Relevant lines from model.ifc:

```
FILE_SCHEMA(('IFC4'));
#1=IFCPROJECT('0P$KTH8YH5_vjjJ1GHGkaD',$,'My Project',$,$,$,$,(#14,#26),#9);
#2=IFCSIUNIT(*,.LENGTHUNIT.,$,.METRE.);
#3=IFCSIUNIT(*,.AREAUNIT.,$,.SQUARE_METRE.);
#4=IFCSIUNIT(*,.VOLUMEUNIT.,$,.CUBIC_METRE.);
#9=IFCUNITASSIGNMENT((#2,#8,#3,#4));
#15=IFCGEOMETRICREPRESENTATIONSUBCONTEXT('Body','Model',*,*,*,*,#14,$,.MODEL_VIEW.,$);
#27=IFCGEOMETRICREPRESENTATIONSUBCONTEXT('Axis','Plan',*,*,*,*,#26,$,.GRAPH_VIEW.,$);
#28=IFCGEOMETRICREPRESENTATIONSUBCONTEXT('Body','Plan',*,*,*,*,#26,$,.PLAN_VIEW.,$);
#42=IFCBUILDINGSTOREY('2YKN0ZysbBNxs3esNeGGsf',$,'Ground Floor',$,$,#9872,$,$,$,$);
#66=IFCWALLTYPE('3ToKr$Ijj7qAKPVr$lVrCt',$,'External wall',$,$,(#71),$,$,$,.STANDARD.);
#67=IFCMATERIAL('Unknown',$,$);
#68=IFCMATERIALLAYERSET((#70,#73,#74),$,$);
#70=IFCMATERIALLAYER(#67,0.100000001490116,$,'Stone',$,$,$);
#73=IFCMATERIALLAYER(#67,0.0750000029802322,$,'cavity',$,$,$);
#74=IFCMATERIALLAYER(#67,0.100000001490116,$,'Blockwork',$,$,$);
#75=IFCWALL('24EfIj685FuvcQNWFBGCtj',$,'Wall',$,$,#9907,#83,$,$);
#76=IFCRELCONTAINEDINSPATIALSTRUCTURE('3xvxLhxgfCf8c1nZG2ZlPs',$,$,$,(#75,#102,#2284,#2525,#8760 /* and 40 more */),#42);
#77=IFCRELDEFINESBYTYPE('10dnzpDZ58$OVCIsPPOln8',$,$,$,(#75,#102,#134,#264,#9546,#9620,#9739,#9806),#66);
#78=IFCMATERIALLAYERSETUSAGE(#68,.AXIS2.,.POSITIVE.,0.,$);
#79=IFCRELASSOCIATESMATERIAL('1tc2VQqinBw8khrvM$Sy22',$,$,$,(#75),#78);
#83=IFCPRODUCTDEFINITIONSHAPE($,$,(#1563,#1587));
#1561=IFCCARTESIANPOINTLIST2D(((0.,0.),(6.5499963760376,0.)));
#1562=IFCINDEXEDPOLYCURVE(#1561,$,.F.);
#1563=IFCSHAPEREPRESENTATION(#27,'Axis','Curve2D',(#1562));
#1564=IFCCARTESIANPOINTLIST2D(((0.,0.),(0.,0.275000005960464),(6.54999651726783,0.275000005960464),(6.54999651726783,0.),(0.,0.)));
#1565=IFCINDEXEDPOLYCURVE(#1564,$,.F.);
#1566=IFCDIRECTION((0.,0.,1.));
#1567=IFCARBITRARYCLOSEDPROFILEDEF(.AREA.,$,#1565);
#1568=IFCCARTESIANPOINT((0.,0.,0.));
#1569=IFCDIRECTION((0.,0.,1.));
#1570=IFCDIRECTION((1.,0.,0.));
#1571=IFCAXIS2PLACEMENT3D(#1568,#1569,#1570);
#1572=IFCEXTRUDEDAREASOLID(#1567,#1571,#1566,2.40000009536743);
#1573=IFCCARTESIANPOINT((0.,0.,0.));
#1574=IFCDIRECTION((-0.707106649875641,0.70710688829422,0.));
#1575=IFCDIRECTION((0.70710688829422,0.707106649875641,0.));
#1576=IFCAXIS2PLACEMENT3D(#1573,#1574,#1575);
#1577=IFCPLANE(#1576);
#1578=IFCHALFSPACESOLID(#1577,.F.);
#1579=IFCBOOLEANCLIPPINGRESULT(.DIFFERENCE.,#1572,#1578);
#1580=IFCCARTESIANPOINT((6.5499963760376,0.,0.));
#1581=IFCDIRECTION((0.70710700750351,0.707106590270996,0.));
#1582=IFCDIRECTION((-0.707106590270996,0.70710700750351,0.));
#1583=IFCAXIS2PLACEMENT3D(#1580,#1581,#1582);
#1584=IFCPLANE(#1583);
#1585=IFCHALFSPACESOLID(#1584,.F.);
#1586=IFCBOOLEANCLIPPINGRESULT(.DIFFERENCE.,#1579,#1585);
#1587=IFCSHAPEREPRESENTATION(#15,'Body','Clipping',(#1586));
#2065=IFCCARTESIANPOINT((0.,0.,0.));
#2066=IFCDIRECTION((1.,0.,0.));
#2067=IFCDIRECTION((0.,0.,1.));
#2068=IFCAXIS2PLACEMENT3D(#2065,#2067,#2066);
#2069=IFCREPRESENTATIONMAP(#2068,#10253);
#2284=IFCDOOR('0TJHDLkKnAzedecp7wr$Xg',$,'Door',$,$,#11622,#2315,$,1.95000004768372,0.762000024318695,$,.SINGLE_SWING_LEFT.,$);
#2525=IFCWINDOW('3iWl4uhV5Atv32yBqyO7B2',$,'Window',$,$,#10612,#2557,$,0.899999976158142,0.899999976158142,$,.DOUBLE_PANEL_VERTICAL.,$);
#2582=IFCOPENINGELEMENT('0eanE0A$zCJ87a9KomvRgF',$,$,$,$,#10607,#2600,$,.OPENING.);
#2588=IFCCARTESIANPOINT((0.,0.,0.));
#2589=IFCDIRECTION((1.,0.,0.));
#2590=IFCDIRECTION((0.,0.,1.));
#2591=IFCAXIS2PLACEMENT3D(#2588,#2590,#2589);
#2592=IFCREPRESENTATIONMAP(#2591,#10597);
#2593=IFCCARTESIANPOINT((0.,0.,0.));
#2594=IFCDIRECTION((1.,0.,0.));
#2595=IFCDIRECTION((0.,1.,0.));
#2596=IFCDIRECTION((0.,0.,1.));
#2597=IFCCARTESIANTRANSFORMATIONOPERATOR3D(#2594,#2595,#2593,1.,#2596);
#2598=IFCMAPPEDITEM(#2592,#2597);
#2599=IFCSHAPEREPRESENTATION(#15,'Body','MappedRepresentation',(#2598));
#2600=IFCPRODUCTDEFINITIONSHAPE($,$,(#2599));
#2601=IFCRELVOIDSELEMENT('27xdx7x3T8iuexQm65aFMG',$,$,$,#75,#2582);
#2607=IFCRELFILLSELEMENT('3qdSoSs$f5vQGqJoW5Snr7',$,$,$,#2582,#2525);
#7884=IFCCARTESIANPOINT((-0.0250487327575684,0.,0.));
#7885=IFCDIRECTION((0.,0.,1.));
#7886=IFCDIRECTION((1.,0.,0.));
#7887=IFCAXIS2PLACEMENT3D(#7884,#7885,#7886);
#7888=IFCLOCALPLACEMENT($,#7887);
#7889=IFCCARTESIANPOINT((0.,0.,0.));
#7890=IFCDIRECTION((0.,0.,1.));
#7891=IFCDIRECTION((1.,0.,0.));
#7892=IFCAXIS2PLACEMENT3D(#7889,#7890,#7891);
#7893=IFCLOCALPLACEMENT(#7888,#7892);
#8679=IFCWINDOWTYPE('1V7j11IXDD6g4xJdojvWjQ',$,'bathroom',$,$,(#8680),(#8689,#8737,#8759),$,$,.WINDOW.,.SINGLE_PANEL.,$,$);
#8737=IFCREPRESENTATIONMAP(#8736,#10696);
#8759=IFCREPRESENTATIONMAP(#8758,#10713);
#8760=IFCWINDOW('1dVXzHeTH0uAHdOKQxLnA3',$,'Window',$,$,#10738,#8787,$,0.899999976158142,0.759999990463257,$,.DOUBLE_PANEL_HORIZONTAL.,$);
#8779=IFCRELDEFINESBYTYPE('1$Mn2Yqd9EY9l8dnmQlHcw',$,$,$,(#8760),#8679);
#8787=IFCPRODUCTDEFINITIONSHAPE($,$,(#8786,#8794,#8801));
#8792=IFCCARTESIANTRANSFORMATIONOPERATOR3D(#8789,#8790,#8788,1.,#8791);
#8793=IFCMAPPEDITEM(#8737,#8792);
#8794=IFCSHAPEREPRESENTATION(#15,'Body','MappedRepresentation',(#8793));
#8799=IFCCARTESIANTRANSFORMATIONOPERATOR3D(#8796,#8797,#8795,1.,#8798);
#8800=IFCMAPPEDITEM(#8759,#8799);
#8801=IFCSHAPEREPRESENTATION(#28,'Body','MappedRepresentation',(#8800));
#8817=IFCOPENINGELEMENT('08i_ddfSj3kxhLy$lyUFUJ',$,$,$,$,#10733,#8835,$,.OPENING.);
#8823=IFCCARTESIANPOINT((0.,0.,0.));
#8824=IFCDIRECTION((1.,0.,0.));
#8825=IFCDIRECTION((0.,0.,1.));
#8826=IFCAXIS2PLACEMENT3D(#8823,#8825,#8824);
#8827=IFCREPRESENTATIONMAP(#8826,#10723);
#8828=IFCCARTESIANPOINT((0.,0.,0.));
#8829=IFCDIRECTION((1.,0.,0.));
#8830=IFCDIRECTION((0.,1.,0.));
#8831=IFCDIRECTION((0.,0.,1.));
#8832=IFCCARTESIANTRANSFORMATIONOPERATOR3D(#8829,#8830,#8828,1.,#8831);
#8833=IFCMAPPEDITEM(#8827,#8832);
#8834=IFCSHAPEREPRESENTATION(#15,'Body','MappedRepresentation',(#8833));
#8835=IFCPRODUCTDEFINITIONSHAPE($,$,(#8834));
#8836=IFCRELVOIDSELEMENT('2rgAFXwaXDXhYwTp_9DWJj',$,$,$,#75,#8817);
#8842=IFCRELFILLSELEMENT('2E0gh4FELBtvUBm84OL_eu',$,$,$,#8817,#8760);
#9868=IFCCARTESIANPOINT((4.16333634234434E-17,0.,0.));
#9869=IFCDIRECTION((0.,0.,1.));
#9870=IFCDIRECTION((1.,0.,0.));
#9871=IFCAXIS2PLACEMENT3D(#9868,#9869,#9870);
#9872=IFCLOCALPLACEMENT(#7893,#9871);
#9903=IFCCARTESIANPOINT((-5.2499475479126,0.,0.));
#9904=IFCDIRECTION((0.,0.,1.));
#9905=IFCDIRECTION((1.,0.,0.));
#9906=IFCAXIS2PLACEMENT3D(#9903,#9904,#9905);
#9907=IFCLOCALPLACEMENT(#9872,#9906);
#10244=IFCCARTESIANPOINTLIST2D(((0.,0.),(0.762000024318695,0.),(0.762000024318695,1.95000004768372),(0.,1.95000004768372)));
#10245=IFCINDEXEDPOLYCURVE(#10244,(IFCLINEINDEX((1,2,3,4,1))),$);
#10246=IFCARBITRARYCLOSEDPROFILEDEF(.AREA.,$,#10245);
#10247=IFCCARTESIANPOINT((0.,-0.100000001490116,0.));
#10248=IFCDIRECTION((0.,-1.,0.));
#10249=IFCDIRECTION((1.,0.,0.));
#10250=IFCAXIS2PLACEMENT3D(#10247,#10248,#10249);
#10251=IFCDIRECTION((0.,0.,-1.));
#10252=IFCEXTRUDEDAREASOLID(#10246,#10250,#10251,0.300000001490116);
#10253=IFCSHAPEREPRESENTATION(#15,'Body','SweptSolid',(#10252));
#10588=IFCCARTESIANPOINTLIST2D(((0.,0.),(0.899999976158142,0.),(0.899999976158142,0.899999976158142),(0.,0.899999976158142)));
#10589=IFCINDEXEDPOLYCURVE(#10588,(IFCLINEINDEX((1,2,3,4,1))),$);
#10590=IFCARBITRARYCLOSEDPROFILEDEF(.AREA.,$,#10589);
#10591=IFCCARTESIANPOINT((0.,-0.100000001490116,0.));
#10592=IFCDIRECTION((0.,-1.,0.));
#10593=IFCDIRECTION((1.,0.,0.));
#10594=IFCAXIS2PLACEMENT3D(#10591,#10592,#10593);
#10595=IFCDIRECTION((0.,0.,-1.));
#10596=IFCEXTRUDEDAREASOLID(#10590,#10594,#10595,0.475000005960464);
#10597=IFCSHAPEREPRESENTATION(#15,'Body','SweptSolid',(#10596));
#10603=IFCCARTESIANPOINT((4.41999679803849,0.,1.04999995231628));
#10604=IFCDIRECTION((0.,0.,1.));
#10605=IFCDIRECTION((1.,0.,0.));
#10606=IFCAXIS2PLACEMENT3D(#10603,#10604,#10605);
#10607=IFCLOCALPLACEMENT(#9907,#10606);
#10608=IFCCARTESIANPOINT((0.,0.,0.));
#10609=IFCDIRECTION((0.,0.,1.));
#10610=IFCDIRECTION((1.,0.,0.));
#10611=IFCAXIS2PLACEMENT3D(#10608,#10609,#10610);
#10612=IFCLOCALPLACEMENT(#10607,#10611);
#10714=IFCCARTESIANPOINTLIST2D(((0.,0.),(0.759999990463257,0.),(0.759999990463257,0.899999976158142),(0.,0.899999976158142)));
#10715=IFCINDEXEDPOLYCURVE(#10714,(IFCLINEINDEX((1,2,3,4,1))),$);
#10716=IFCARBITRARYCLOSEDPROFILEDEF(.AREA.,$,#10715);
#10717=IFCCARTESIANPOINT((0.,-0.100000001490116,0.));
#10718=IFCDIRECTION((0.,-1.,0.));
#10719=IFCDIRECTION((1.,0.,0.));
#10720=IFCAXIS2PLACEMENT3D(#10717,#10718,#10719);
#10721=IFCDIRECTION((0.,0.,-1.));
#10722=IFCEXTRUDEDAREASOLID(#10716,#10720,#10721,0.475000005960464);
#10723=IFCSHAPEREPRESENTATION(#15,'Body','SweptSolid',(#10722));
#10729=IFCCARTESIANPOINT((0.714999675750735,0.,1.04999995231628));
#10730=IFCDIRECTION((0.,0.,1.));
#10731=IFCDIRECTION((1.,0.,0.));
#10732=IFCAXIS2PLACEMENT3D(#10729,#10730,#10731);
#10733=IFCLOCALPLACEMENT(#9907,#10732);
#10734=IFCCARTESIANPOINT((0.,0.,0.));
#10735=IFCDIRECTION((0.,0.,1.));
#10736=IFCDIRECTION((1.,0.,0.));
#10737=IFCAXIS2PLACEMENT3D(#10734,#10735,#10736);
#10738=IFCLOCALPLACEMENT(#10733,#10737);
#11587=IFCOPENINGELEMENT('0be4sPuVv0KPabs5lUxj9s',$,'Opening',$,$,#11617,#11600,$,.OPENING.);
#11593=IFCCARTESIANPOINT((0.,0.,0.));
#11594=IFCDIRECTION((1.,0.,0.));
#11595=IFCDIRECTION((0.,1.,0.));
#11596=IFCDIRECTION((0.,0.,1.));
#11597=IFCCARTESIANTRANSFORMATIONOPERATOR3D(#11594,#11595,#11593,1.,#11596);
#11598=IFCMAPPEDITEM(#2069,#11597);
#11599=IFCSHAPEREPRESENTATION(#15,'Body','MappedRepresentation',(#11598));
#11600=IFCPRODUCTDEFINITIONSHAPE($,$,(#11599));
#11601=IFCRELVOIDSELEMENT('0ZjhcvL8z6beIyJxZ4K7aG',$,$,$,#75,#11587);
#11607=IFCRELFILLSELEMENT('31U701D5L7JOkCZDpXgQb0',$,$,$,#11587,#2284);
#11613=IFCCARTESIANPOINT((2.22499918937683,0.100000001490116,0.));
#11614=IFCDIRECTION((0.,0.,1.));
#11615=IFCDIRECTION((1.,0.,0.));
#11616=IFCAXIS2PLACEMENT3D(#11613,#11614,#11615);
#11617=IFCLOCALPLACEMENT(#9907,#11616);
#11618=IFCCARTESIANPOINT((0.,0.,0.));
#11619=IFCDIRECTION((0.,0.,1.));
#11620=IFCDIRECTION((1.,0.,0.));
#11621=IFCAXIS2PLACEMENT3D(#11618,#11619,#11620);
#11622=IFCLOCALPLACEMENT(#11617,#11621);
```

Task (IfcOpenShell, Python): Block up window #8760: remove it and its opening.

```python
import ifcopenshell
import ifcopenshell.api.feature
import ifcopenshell.api.root
import ifcopenshell.geom
import ifcopenshell.util.shape

model = ifcopenshell.open("model.ifc")
settings = ifcopenshell.geom.settings()


def volume(element):
    """Net volume in cubic metres, openings subtracted."""
    shape = ifcopenshell.geom.create_shape(settings, element)
    return ifcopenshell.util.shape.get_volume(shape.geometry)


window = model.by_guid("1dVXzHeTH0uAHdOKQxLnA3")
opening = window.FillsVoids[0].RelatingOpeningElement
wall = opening.VoidsElements[0].RelatingBuildingElement
before = volume(wall)

ifcopenshell.api.root.remove_product(model, product=window)
ifcopenshell.api.feature.remove_feature(model, feature=opening)

after = volume(wall)

print(f"wall volume {before:.3f} -> {after:.3f} m3")

model.write("model_rev.ifc")
```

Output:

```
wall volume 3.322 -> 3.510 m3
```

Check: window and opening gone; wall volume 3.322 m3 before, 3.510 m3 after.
